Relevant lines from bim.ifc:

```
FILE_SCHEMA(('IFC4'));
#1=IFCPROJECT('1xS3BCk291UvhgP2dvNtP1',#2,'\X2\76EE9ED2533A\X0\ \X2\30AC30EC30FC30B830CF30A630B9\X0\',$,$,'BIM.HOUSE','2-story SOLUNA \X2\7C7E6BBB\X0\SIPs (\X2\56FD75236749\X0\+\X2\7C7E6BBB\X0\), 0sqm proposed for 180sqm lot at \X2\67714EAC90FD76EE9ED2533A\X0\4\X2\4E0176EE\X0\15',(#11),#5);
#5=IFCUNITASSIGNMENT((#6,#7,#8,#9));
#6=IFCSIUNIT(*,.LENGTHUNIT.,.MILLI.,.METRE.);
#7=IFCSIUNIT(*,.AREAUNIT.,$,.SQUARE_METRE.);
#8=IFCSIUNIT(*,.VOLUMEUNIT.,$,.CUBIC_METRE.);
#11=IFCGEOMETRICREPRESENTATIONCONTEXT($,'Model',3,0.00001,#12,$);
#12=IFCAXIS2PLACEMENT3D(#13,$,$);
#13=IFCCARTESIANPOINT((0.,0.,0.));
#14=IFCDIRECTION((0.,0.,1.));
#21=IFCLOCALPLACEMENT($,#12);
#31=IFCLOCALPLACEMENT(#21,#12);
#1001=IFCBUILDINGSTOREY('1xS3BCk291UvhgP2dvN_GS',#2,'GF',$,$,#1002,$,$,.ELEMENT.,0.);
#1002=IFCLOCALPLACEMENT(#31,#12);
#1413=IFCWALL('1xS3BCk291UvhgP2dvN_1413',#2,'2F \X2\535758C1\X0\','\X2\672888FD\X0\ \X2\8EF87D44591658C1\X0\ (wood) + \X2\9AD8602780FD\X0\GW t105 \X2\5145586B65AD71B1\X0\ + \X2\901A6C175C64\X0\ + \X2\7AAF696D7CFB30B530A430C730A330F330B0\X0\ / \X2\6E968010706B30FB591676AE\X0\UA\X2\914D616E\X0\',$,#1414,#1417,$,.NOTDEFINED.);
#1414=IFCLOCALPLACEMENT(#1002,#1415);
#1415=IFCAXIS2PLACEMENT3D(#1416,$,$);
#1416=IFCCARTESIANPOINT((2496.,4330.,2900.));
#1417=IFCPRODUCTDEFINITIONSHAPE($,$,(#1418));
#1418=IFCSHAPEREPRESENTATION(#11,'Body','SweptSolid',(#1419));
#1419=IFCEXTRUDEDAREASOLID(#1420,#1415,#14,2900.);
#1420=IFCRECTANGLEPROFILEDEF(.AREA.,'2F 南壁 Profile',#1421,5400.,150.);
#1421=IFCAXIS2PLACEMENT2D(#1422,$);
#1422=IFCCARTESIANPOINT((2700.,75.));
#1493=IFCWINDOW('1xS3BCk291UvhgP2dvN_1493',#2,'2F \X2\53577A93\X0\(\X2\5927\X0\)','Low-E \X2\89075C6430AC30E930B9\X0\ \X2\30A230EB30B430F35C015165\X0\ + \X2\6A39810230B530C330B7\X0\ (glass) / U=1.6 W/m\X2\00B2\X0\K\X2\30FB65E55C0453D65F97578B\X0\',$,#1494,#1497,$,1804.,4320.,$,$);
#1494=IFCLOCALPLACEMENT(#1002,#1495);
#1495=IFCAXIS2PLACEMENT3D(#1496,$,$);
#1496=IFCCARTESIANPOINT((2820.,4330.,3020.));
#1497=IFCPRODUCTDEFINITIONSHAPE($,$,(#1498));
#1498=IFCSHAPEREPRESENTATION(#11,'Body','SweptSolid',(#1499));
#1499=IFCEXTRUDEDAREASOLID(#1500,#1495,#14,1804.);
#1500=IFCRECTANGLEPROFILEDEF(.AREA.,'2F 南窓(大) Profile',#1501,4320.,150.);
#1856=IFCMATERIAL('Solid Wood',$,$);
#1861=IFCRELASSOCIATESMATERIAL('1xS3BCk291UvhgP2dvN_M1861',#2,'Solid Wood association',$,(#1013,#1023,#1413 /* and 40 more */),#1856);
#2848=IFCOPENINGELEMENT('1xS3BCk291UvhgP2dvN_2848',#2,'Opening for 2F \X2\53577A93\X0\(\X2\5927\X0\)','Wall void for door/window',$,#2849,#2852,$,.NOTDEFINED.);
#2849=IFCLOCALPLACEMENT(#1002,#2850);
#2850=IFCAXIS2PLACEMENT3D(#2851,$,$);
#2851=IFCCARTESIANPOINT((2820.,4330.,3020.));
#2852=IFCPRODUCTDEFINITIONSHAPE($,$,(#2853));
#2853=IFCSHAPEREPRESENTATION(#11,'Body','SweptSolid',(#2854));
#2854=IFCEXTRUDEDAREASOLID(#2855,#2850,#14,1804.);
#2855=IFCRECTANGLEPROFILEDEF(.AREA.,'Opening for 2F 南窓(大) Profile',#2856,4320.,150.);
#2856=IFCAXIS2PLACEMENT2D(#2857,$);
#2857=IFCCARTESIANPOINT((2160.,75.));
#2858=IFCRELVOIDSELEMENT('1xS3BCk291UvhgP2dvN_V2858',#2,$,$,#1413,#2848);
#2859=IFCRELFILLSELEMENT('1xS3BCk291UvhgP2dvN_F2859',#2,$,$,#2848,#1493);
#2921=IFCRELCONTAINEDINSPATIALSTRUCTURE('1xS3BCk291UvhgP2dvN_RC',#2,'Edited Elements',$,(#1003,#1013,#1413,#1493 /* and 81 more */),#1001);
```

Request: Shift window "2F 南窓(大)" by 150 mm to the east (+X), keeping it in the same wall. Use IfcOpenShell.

```python
import ifcopenshell
import ifcopenshell.api.geometry
import ifcopenshell.util.placement
import ifcopenshell.util.unit

model = ifcopenshell.open("bim.ifc")
unit_scale = ifcopenshell.util.unit.calculate_unit_scale(model)

window = model.by_guid("1xS3BCk291UvhgP2dvN_1493")
opening = window.FillsVoids[0].RelatingOpeningElement
wall = opening.VoidsElements[0].RelatingBuildingElement

wall_matrix = ifcopenshell.util.placement.get_local_placement(wall.ObjectPlacement)
shift = wall_matrix[:3, 0] * 0.15 / unit_scale
before = ifcopenshell.util.placement.get_local_placement(window.ObjectPlacement)[:3, 3].copy()

# The window is not placed relative to its opening, so move both.
for product in (opening, window):
    matrix = ifcopenshell.util.placement.get_local_placement(product.ObjectPlacement)
    matrix[:3, 3] += shift
    ifcopenshell.api.geometry.edit_object_placement(model, product=product, matrix=matrix, is_si=False)

after = ifcopenshell.util.placement.get_local_placement(window.ObjectPlacement)[:3, 3]
print("window moved by", (after - before).round(3) + 0.0)

model.write("bim_updated.ifc")
```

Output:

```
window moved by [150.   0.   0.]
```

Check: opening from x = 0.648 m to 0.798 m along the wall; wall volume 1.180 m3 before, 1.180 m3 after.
